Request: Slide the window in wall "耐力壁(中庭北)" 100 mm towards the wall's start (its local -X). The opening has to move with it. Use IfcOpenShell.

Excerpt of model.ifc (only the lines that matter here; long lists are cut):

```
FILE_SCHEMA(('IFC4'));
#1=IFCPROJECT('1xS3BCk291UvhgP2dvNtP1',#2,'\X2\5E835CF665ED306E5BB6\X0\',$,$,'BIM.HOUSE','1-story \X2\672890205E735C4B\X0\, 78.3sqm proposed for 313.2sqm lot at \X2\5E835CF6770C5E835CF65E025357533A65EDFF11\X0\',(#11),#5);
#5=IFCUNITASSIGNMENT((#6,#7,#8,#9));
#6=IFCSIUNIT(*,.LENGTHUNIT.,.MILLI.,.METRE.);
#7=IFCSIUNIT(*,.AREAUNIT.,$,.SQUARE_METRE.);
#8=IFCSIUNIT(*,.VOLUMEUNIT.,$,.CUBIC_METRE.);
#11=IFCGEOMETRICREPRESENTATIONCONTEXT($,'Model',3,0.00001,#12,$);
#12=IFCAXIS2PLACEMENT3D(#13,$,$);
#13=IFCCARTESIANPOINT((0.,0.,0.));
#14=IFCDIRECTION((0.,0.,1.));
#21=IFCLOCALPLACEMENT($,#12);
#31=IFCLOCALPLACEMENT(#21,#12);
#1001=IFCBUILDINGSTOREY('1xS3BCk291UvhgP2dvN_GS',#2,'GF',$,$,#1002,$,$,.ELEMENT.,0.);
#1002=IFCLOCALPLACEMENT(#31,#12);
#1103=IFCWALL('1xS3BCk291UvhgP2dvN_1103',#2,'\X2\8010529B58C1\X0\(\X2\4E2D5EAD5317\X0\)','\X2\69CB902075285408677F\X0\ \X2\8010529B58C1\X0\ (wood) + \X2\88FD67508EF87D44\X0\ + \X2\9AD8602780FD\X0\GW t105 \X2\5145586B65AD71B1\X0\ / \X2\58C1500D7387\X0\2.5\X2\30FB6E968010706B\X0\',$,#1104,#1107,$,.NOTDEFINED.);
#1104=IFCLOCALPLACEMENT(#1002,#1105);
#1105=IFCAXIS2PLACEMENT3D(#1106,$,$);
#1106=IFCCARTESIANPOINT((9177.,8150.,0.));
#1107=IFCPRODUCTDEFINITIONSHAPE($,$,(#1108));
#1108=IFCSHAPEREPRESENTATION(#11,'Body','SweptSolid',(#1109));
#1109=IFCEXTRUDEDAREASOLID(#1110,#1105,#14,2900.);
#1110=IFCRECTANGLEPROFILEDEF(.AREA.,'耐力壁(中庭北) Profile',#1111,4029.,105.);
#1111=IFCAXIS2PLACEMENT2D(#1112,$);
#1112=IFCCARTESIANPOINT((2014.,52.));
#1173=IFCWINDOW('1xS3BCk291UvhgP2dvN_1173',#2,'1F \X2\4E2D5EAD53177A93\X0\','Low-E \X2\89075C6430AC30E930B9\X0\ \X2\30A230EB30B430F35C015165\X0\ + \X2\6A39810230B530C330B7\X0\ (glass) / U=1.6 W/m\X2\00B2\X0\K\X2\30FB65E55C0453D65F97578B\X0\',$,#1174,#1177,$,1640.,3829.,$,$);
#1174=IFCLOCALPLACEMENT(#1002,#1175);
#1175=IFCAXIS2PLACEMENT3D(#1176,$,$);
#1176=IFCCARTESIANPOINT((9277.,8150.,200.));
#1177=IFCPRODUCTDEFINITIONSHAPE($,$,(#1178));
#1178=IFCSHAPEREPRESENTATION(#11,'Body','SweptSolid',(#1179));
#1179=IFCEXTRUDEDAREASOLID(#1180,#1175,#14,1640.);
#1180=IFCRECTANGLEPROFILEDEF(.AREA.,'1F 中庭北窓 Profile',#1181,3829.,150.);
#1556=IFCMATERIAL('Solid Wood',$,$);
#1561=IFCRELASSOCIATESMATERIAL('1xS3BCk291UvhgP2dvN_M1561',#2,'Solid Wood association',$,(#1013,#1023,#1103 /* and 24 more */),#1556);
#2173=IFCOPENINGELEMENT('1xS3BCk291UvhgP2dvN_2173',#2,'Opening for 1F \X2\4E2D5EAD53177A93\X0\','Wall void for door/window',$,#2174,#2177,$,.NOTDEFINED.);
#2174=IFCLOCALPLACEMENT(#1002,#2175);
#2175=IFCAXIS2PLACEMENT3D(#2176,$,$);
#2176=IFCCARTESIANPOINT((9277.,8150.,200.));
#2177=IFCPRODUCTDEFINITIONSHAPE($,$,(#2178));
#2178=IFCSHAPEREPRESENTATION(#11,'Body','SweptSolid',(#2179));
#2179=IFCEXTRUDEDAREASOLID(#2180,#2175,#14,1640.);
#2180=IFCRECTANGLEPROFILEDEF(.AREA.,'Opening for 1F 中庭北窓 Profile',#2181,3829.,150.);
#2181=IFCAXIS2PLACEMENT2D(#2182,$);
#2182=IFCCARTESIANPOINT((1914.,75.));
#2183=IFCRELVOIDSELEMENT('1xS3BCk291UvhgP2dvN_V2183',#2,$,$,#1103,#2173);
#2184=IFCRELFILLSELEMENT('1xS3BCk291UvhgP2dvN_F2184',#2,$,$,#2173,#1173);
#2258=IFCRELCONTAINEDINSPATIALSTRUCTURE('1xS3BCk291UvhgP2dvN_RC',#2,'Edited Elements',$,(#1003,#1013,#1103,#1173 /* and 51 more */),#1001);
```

```python
import ifcopenshell
import ifcopenshell.api.geometry
import ifcopenshell.util.placement

model = ifcopenshell.open("model.ifc")

window = model.by_guid("1xS3BCk291UvhgP2dvN_1173")
opening = window.FillsVoids[0].RelatingOpeningElement
wall = opening.VoidsElements[0].RelatingBuildingElement

wall_matrix = ifcopenshell.util.placement.get_local_placement(wall.ObjectPlacement)
shift = wall_matrix[:3, 0] * -100.0
before = ifcopenshell.util.placement.get_local_placement(window.ObjectPlacement)[:3, 3].copy()

# The window is not placed relative to its opening, so move both.
for product in (opening, window):
    matrix = ifcopenshell.util.placement.get_local_placement(product.ObjectPlacement)
    matrix[:3, 3] += shift
    ifcopenshell.api.geometry.edit_object_placement(model, product=product, matrix=matrix, is_si=False)

after = ifcopenshell.util.placement.get_local_placement(window.ObjectPlacement)[:3, 3]
print("window moved by", (after - before).round(3) + 0.0)

model.write("model_updated.ifc")
```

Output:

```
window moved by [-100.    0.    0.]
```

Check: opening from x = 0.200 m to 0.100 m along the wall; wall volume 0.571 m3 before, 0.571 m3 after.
